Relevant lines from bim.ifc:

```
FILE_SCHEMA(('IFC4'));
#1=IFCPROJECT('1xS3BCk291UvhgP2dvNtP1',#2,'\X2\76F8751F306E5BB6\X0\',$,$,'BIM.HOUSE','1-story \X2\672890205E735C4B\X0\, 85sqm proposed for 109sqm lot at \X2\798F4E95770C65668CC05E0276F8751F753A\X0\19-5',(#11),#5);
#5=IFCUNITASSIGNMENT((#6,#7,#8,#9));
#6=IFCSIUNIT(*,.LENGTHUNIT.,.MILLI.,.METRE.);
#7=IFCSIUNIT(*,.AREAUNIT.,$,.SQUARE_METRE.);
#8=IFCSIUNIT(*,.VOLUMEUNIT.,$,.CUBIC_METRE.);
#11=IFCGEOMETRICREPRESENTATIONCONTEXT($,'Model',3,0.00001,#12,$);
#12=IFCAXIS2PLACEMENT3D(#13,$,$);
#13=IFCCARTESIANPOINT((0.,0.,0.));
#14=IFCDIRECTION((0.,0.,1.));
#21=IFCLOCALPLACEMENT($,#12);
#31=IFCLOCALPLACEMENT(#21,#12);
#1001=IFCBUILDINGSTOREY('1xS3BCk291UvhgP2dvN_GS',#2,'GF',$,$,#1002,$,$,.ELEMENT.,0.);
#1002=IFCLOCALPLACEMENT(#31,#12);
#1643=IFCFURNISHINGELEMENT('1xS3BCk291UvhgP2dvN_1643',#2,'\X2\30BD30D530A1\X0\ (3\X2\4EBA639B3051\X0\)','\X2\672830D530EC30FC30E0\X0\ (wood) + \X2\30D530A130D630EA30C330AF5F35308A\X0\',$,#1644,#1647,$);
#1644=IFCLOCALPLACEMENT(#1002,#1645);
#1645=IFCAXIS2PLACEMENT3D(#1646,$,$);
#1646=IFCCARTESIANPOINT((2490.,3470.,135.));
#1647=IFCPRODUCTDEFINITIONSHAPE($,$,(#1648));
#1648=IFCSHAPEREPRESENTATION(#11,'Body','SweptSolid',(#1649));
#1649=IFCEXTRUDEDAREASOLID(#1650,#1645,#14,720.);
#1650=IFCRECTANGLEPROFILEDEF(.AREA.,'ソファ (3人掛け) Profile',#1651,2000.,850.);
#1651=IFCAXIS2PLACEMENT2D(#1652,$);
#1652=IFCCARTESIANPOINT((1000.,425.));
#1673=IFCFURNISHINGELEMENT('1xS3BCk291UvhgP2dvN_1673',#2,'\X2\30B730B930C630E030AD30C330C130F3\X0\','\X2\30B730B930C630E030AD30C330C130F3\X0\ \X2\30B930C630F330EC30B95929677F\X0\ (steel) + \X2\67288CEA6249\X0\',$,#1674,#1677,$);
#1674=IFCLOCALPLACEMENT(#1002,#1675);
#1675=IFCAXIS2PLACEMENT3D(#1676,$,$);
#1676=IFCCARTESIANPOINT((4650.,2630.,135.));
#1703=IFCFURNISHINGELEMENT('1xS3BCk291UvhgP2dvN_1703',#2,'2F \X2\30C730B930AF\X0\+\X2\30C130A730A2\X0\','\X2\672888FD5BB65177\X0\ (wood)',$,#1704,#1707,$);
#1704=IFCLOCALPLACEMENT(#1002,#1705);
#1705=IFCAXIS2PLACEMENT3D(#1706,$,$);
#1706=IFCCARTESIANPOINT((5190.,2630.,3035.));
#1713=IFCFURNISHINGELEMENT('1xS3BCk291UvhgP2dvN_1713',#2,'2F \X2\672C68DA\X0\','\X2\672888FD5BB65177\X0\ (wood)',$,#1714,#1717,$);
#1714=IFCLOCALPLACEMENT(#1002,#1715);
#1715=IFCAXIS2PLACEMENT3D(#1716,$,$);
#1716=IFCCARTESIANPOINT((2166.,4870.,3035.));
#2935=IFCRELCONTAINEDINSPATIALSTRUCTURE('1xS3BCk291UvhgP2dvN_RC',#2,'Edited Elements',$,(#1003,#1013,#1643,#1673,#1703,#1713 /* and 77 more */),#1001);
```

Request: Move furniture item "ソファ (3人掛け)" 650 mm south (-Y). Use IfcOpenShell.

```python
import ifcopenshell
import ifcopenshell.api.geometry
import ifcopenshell.util.placement

model = ifcopenshell.open("bim.ifc")

item = model.by_id(1643)
matrix = ifcopenshell.util.placement.get_local_placement(item.ObjectPlacement)
matrix[1, 3] -= 650.0
ifcopenshell.api.geometry.edit_object_placement(model, product=item, matrix=matrix, is_si=False)

print(ifcopenshell.util.placement.get_local_placement(item.ObjectPlacement).round(3) + 0.0)

model.write("bim_edited.ifc")
```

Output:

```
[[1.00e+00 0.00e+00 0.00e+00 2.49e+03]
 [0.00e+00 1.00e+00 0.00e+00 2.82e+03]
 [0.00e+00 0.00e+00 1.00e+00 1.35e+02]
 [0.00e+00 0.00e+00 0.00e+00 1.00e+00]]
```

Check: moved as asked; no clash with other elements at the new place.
